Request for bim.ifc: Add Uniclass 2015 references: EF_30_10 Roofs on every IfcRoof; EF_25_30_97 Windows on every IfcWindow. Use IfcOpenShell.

First a look at what the model holds.

```python
import ifcopenshell

model = ifcopenshell.open("bim.ifc")
print(model.schema)
print("classifications:", [c.Name for c in model.by_type("IfcClassification")])
for ifc_class in ("IfcDoor", "IfcRoof", "IfcStair", "IfcWall", "IfcWindow"):
    print(ifc_class, len(model.by_type(ifc_class)))
```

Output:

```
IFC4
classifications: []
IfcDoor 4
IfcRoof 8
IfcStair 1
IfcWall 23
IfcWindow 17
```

```python
import ifcopenshell
import ifcopenshell.api.classification

model = ifcopenshell.open("bim.ifc")

system = ifcopenshell.api.classification.add_classification(model, classification="Uniclass 2015")

codes = {
    "IfcRoof": ("EF_30_10", "Roofs"),
    "IfcWindow": ("EF_25_30_97", "Windows"),
}
for ifc_class, (code, name) in codes.items():
    products = model.by_type(ifc_class)
    ifcopenshell.api.classification.add_reference(
        model, products=products, classification=system, identification=code, name=name
    )
    print(code, len(products))

model.write("bim_edited.ifc")
```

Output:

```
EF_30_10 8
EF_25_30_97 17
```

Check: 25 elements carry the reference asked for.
